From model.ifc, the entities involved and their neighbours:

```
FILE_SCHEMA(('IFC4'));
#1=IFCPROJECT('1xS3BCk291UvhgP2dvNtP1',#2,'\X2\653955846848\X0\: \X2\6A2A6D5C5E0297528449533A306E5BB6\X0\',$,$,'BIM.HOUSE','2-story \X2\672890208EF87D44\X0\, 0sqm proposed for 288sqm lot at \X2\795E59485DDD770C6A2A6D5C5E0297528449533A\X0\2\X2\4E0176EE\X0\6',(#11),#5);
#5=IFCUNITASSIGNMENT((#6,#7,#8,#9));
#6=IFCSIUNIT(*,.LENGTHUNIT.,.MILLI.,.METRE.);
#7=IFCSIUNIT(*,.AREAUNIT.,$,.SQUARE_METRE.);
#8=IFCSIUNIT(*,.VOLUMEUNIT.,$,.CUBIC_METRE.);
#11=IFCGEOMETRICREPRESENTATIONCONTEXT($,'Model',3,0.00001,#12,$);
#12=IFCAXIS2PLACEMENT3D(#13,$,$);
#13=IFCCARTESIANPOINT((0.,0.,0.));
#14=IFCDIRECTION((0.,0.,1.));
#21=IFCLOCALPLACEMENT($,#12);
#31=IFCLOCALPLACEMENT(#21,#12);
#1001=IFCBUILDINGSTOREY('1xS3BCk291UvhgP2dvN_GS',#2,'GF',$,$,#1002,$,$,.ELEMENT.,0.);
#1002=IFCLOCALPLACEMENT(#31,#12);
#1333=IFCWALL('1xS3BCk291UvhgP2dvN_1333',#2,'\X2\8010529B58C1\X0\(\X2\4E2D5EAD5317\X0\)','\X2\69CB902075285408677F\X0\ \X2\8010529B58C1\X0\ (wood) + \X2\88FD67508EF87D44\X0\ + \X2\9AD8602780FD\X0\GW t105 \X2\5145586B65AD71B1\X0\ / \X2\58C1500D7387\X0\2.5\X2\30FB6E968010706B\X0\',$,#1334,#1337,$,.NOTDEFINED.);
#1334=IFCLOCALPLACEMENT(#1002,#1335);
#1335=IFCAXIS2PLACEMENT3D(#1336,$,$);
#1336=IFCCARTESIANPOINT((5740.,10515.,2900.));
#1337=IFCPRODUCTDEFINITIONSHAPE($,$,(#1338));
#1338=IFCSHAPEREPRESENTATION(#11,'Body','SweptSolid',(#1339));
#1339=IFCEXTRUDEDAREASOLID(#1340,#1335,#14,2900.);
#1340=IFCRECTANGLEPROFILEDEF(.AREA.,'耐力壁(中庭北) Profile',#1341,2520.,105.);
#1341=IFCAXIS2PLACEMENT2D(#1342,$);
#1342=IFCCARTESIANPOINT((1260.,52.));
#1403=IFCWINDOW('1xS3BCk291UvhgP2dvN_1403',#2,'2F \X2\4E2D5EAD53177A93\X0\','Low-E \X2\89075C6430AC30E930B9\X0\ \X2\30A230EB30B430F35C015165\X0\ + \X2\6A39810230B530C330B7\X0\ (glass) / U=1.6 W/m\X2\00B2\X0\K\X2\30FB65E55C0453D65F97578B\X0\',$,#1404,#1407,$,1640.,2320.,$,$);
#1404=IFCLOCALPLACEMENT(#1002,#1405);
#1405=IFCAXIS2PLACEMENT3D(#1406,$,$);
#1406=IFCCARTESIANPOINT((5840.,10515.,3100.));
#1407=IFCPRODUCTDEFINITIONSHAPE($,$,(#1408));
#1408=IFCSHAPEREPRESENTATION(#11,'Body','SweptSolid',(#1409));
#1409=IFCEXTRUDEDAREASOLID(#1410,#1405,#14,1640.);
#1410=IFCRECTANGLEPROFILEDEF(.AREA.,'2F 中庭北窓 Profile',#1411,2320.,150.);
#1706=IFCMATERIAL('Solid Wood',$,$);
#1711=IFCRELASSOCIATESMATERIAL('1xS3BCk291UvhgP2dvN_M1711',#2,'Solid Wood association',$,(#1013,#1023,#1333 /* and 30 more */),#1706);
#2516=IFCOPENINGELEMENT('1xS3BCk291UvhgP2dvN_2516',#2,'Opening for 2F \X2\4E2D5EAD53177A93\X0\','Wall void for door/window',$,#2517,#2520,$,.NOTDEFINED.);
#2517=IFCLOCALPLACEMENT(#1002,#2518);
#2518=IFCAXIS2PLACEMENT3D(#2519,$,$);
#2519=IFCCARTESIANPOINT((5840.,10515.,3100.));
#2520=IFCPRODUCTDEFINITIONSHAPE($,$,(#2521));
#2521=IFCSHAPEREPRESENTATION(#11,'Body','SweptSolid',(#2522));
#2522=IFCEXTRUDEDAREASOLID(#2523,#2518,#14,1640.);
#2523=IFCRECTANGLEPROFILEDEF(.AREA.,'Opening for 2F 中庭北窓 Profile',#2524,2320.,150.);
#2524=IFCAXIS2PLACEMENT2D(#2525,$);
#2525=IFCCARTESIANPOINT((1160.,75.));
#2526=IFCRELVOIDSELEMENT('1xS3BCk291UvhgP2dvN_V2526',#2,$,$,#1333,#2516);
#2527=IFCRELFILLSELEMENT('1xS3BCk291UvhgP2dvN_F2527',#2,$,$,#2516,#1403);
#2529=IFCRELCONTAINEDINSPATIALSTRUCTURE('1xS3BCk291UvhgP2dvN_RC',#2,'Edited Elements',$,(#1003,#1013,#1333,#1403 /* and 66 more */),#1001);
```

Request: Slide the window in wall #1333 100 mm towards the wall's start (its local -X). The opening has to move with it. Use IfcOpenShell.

```python
import ifcopenshell
import ifcopenshell.api.geometry
import ifcopenshell.util.placement

model = ifcopenshell.open("model.ifc")

window = model.by_guid("1xS3BCk291UvhgP2dvN_1403")
opening = window.FillsVoids[0].RelatingOpeningElement
wall = opening.VoidsElements[0].RelatingBuildingElement

wall_matrix = ifcopenshell.util.placement.get_local_placement(wall.ObjectPlacement)
shift = wall_matrix[:3, 0] * -100.0
before = ifcopenshell.util.placement.get_local_placement(window.ObjectPlacement)[:3, 3].copy()

# The window is not placed relative to its opening, so move both.
for product in (opening, window):
    matrix = ifcopenshell.util.placement.get_local_placement(product.ObjectPlacement)
    matrix[:3, 3] += shift
    ifcopenshell.api.geometry.edit_object_placement(model, product=product, matrix=matrix, is_si=False)

after = ifcopenshell.util.placement.get_local_placement(window.ObjectPlacement)[:3, 3]
print("window moved by", (after - before).round(3) + 0.0)

model.write("model_updated.ifc")
```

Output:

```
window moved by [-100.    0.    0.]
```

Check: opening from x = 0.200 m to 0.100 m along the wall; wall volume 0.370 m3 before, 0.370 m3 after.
